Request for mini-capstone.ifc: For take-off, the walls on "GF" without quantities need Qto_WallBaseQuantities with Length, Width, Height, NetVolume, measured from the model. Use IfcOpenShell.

First a look at what the model holds.

```python
import ifcopenshell
import ifcopenshell.util.element
import ifcopenshell.util.unit

model = ifcopenshell.open("mini-capstone.ifc")
print(model.schema)
for unit_type in ("LENGTHUNIT", "AREAUNIT", "VOLUMEUNIT"):
    print(unit_type, ifcopenshell.util.unit.calculate_unit_scale(model, unit_type))
storey = next(s for s in model.by_type("IfcBuildingStorey") if s.Name == "GF")
walls = [e for e in ifcopenshell.util.element.get_decomposition(storey) if e.is_a("IfcWall")]
for e in sorted(walls, key=lambda e: e.id()):
    print(e.id(), e.is_a(), e.Name, list(ifcopenshell.util.element.get_psets(e, qtos_only=True)), sep=" | ")
```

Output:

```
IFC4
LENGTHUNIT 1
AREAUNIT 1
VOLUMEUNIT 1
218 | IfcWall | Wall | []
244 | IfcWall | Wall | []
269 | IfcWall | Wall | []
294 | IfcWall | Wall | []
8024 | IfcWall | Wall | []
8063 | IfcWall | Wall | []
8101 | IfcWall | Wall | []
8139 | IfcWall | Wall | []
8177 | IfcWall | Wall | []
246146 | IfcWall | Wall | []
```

```python
import ifcopenshell
import ifcopenshell.api.pset
import ifcopenshell.geom
import ifcopenshell.util.element
import ifcopenshell.util.shape
import ifcopenshell.util.unit

model = ifcopenshell.open("mini-capstone.ifc")
unit_scale = ifcopenshell.util.unit.calculate_unit_scale(model)
volume_scale = ifcopenshell.util.unit.calculate_unit_scale(model, "VOLUMEUNIT")
settings = ifcopenshell.geom.settings()

storey = next(s for s in model.by_type("IfcBuildingStorey") if s.Name == "GF")
walls = [e for e in ifcopenshell.util.element.get_decomposition(storey) if e.is_a("IfcWall")]

for e in sorted(walls, key=lambda e: e.id()):
    if ifcopenshell.util.element.get_psets(e, qtos_only=True, should_inherit=False):
        continue
    # Geometry comes back in metres, in the element's own axes.
    shape = ifcopenshell.geom.create_shape(settings, e)
    values = {
        "Length": ifcopenshell.util.shape.get_x(shape.geometry) / unit_scale,
        "Width": ifcopenshell.util.shape.get_y(shape.geometry) / unit_scale,
        "Height": ifcopenshell.util.shape.get_z(shape.geometry) / unit_scale,
        "NetVolume": ifcopenshell.util.shape.get_volume(shape.geometry) / volume_scale,
    }
    qto = ifcopenshell.api.pset.add_qto(model, product=e, name="Qto_WallBaseQuantities")
    ifcopenshell.api.pset.edit_qto(model, qto=qto, properties=values)
    print(e.id(), {k: round(v, 3) for k, v in values.items()})

model.write("mini-capstone_v2.ifc")
```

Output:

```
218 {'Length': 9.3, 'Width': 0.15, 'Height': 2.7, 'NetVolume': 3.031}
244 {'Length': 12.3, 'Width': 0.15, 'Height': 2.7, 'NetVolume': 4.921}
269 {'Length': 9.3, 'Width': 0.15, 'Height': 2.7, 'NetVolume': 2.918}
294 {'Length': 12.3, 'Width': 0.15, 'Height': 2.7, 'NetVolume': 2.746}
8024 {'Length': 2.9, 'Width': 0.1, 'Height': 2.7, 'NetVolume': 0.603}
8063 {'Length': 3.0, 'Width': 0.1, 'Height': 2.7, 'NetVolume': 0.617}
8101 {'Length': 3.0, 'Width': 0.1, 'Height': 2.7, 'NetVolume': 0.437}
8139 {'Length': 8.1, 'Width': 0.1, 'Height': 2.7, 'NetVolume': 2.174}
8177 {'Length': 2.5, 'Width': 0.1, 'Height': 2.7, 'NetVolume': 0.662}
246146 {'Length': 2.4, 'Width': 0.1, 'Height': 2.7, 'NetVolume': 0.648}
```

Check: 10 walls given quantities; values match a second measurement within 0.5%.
